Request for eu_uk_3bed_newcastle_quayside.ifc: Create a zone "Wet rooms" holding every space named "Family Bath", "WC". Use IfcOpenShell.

First a look at what the model holds.

```python
import ifcopenshell

model = ifcopenshell.open("eu_uk_3bed_newcastle_quayside.ifc")
print(model.schema)
seen = {}
for space in model.by_type("IfcSpace"):
    seen[space.LongName] = seen.get(space.LongName, 0) + 1
for name, count in sorted(seen.items(), key=str):
    print(count, "x", name)
print("zones:", [z.Name for z in model.by_type("IfcZone")][:20])
```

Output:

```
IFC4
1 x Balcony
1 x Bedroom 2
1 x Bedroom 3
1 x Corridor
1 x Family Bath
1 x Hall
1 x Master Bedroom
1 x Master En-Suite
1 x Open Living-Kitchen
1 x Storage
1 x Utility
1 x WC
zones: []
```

```python
import ifcopenshell
import ifcopenshell.api.group
import ifcopenshell.api.root

model = ifcopenshell.open("eu_uk_3bed_newcastle_quayside.ifc")

names = {"Family Bath", "WC"}
spaces = [s for s in model.by_type("IfcSpace") if s.LongName in names]

zone = ifcopenshell.api.root.create_entity(model, ifc_class="IfcZone", name="Wet rooms")
ifcopenshell.api.group.assign_group(model, products=spaces, group=zone)
print(len(spaces), "spaces in", zone.Name)

model.write("eu_uk_3bed_newcastle_quayside_updated.ifc")
```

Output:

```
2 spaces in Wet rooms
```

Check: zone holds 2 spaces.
